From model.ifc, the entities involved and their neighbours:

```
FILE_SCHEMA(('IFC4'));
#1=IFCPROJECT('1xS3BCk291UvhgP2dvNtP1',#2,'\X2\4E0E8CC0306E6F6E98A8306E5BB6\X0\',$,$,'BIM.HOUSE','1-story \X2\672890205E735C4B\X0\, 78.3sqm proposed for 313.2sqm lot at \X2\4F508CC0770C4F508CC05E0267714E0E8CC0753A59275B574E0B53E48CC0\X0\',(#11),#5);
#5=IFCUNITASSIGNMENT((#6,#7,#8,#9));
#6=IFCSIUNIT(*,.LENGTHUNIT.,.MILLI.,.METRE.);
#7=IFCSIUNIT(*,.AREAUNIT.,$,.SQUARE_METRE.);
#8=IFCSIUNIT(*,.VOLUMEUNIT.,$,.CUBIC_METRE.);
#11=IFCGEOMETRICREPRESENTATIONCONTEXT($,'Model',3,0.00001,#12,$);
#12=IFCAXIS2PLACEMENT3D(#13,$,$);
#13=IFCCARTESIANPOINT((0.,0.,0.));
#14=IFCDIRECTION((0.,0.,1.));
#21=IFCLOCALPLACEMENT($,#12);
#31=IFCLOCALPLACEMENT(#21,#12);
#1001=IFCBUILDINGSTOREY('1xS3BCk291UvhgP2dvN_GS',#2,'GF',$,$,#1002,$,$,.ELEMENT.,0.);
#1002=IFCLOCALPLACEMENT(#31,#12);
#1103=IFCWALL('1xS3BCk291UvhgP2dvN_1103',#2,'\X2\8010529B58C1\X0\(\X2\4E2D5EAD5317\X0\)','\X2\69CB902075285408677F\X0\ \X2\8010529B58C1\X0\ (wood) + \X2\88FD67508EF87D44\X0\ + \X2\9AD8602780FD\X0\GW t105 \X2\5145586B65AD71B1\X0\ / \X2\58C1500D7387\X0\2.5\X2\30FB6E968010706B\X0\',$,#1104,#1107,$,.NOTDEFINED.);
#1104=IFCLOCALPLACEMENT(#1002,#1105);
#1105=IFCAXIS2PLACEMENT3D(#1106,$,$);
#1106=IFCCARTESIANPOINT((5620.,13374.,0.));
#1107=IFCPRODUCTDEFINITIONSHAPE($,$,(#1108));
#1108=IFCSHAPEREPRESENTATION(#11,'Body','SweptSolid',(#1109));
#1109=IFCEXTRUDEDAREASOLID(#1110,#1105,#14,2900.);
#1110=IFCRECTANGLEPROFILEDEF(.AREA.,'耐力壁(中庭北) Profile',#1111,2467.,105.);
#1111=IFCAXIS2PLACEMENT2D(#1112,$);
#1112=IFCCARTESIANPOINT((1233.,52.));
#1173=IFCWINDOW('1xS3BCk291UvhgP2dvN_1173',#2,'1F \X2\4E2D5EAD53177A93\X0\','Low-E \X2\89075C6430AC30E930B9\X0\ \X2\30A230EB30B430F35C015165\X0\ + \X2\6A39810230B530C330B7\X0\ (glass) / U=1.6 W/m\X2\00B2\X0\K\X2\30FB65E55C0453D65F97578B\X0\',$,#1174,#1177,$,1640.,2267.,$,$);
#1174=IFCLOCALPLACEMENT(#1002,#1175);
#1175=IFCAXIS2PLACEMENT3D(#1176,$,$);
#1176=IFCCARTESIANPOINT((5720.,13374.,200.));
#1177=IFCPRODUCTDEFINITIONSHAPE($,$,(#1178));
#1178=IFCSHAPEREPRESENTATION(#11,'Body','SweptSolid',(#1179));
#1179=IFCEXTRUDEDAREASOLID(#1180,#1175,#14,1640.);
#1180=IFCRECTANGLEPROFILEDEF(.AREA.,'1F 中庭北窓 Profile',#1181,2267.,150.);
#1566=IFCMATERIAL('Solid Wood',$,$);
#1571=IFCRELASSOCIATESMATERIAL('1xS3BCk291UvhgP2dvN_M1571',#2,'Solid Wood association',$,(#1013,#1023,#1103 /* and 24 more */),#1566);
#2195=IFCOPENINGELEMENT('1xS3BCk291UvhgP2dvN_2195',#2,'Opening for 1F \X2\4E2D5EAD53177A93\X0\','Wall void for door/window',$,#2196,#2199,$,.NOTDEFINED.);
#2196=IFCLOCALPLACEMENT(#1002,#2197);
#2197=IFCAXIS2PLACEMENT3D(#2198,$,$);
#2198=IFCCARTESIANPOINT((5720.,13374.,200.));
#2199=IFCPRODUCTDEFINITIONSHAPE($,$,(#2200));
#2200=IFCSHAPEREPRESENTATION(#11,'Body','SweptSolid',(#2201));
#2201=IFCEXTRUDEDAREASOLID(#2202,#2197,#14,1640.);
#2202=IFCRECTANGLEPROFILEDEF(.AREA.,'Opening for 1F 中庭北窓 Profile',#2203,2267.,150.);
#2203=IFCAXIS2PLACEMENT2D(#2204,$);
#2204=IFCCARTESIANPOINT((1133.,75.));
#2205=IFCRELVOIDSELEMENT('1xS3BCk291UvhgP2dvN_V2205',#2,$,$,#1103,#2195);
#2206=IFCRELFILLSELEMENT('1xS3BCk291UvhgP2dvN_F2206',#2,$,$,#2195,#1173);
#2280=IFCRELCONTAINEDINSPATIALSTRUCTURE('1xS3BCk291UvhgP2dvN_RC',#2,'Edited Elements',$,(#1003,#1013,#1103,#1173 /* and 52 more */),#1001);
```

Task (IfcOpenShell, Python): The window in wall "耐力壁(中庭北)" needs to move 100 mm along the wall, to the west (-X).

```python
import ifcopenshell
import ifcopenshell.api.geometry
import ifcopenshell.util.placement

model = ifcopenshell.open("model.ifc")

window = model.by_guid("1xS3BCk291UvhgP2dvN_1173")
opening = window.FillsVoids[0].RelatingOpeningElement
wall = opening.VoidsElements[0].RelatingBuildingElement

wall_matrix = ifcopenshell.util.placement.get_local_placement(wall.ObjectPlacement)
shift = wall_matrix[:3, 0] * -100.0
before = ifcopenshell.util.placement.get_local_placement(window.ObjectPlacement)[:3, 3].copy()

# The window is not placed relative to its opening, so move both.
for product in (opening, window):
    matrix = ifcopenshell.util.placement.get_local_placement(product.ObjectPlacement)
    matrix[:3, 3] += shift
    ifcopenshell.api.geometry.edit_object_placement(model, product=product, matrix=matrix, is_si=False)

after = ifcopenshell.util.placement.get_local_placement(window.ObjectPlacement)[:3, 3]
print("window moved by", (after - before).round(3) + 0.0)

model.write("model-out.ifc")
```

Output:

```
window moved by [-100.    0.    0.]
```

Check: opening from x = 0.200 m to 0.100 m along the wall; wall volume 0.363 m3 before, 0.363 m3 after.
